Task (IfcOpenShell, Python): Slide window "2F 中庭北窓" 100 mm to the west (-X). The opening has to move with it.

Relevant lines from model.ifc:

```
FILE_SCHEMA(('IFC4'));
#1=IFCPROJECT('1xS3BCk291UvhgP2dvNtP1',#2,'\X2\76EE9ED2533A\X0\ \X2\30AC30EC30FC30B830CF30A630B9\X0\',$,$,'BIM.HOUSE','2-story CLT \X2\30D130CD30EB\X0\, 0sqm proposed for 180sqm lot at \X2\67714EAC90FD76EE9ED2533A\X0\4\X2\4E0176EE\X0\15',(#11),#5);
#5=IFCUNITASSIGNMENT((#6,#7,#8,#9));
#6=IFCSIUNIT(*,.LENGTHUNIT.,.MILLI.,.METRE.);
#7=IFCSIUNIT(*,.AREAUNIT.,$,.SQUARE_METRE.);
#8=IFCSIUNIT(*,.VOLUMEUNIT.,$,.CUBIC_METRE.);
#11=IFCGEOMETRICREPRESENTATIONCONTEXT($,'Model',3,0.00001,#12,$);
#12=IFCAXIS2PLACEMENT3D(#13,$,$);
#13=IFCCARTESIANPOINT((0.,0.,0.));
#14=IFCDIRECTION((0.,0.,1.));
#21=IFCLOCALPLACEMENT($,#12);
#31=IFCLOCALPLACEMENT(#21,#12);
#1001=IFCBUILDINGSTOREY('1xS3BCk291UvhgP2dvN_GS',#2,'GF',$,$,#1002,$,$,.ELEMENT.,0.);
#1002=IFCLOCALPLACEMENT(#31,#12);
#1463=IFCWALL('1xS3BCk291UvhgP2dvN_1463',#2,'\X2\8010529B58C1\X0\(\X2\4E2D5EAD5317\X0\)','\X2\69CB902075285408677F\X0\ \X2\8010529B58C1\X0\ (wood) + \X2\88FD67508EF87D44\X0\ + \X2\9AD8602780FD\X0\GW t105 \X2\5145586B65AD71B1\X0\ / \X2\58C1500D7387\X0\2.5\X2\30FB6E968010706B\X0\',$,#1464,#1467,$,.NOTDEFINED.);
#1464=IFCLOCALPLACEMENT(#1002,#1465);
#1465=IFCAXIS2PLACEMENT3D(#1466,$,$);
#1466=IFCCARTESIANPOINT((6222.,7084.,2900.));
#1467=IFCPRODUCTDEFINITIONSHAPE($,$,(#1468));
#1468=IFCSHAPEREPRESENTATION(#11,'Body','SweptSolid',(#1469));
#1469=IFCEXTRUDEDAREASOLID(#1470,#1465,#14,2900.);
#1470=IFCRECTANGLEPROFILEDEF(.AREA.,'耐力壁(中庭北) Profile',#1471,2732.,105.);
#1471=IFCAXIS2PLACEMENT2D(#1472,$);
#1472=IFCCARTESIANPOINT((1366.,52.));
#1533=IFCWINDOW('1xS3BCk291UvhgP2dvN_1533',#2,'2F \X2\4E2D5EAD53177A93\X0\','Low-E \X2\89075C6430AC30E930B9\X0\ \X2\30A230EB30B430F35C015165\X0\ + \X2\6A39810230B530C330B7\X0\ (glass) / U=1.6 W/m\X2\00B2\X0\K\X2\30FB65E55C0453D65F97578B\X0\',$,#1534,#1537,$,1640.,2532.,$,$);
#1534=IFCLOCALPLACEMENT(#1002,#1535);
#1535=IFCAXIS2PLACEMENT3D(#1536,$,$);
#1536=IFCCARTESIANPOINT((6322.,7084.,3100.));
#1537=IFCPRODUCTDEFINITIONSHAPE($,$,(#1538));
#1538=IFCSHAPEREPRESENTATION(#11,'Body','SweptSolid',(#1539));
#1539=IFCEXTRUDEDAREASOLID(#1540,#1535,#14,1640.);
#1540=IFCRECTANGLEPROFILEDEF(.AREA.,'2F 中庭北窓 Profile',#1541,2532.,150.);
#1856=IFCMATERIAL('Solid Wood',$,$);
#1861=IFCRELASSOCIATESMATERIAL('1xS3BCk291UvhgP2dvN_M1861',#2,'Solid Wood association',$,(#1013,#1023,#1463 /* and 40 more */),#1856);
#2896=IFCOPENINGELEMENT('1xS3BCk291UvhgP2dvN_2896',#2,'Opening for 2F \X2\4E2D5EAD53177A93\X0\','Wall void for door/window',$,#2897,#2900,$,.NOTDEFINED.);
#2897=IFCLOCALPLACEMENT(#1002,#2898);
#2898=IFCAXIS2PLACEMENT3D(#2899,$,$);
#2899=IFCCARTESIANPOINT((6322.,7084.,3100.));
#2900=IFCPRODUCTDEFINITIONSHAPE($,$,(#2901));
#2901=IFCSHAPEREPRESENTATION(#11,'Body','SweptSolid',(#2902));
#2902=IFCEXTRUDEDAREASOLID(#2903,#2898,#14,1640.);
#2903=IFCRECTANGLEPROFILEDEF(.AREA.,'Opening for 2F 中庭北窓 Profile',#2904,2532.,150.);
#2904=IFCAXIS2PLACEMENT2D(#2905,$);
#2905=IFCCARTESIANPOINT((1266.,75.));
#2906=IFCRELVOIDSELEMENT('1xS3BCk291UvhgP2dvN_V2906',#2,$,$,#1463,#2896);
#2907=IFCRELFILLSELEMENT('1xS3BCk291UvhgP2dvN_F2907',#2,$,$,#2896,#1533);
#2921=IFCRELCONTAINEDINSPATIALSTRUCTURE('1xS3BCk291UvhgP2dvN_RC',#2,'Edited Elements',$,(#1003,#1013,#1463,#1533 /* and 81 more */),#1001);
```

```python
import ifcopenshell
import ifcopenshell.api.geometry
import ifcopenshell.util.placement

model = ifcopenshell.open("model.ifc")

window = model.by_id(1533)
opening = window.FillsVoids[0].RelatingOpeningElement
wall = opening.VoidsElements[0].RelatingBuildingElement

wall_matrix = ifcopenshell.util.placement.get_local_placement(wall.ObjectPlacement)
shift = wall_matrix[:3, 0] * -100.0
before = ifcopenshell.util.placement.get_local_placement(window.ObjectPlacement)[:3, 3].copy()

# The window is not placed relative to its opening, so move both.
for product in (opening, window):
    matrix = ifcopenshell.util.placement.get_local_placement(product.ObjectPlacement)
    matrix[:3, 3] += shift
    ifcopenshell.api.geometry.edit_object_placement(model, product=product, matrix=matrix, is_si=False)

after = ifcopenshell.util.placement.get_local_placement(window.ObjectPlacement)[:3, 3]
print("window moved by", (after - before).round(3) + 0.0)

model.write("model_rev.ifc")
```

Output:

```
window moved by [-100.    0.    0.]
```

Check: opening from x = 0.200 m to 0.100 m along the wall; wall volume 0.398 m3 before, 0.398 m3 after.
